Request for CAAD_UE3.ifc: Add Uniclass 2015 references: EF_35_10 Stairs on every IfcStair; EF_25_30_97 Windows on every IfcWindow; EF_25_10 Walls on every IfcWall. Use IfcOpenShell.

First a look at what the model holds.

```python
import ifcopenshell

model = ifcopenshell.open("CAAD_UE3.ifc")
print(model.schema)
print("classifications:", [c.Name for c in model.by_type("IfcClassification")])
for ifc_class in ("IfcDoor", "IfcRoof", "IfcStair", "IfcWall", "IfcWindow"):
    print(ifc_class, len(model.by_type(ifc_class)))
```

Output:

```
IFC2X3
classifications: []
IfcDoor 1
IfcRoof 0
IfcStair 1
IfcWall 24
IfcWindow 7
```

```python
import ifcopenshell
import ifcopenshell.api.classification

model = ifcopenshell.open("CAAD_UE3.ifc")

# IFC2X3 requires Source and Edition and has no link from the project to the system.
system = model.create_entity("IfcClassification", Source="NBS", Edition="2015", Name="Uniclass 2015")

codes = {
    "IfcStair": ("EF_35_10", "Stairs"),
    "IfcWindow": ("EF_25_30_97", "Windows"),
    "IfcWall": ("EF_25_10", "Walls"),
}
for ifc_class, (code, name) in codes.items():
    products = model.by_type(ifc_class)
    ifcopenshell.api.classification.add_reference(
        model, products=products, classification=system, identification=code, name=name
    )
    print(code, len(products))

model.write("CAAD_UE3_edited.ifc")
```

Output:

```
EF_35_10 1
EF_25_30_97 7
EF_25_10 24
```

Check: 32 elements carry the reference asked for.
